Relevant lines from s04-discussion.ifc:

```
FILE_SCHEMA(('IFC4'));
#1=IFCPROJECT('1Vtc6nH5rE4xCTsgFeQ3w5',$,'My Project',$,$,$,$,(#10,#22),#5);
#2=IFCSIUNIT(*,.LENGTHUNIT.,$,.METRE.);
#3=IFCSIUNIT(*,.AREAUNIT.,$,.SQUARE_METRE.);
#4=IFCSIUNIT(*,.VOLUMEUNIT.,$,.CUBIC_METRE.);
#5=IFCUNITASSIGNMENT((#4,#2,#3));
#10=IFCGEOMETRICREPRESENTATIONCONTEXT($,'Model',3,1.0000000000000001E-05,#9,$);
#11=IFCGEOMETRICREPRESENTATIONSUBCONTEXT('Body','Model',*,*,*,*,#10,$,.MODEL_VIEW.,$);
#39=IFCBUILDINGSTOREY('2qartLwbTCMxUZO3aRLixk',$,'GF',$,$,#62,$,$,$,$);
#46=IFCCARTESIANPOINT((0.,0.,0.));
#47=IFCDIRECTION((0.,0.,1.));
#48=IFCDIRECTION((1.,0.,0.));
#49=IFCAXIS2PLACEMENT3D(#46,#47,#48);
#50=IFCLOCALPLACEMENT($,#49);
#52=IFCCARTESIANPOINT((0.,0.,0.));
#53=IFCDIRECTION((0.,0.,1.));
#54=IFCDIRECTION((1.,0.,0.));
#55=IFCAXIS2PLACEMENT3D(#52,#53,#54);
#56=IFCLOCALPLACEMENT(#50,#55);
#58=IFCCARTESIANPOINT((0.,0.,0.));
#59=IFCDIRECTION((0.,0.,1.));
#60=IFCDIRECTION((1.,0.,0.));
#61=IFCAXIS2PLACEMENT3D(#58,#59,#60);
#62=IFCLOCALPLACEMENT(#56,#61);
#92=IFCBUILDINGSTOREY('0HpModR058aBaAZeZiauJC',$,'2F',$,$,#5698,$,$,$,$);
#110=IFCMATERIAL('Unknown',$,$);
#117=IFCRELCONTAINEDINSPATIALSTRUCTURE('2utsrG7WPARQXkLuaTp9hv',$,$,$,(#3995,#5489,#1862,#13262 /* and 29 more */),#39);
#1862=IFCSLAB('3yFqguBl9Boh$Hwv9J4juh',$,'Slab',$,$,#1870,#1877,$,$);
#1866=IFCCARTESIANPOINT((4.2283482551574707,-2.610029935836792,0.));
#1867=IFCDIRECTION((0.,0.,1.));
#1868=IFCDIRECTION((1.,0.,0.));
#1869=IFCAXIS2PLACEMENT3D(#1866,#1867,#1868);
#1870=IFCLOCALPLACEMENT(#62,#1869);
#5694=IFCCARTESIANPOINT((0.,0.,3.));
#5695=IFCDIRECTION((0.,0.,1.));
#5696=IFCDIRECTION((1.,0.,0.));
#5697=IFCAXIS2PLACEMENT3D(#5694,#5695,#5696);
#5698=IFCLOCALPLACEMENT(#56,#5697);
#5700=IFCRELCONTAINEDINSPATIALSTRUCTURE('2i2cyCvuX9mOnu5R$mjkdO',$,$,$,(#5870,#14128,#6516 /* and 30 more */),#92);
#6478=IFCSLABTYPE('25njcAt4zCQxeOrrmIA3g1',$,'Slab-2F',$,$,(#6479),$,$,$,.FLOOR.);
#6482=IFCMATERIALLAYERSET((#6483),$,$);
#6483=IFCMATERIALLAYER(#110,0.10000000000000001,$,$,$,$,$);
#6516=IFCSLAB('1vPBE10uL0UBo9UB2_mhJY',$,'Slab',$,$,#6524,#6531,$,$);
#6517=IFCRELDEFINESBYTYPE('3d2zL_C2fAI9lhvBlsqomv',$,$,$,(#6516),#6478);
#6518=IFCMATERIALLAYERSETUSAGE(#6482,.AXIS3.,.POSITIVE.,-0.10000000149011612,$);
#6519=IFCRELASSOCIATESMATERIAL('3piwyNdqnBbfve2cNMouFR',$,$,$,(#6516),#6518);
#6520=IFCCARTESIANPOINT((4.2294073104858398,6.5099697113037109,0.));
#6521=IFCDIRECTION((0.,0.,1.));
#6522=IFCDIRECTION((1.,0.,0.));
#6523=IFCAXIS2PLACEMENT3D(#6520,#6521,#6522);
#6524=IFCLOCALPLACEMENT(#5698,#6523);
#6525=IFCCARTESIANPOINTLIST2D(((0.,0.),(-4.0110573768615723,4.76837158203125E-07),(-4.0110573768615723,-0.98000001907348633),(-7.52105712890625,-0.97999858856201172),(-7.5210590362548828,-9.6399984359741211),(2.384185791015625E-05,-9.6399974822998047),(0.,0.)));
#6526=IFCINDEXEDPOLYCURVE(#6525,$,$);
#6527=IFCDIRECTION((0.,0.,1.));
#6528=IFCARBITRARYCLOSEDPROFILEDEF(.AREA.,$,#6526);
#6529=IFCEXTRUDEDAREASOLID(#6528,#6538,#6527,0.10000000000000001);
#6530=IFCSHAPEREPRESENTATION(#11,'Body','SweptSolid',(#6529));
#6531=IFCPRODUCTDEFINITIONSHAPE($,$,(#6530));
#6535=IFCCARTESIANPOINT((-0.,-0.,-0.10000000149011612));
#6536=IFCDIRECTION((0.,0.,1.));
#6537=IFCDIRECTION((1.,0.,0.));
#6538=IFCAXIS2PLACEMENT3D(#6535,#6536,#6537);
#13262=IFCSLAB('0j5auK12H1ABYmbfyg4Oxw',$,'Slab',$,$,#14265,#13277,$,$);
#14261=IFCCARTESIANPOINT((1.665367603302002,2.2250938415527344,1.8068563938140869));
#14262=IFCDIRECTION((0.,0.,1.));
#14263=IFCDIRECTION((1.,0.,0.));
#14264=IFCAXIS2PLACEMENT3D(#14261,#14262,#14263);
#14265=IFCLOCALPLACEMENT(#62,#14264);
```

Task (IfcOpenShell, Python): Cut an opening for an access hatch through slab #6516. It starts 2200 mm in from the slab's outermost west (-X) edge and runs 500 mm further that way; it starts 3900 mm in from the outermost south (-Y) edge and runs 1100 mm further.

```python
import numpy as np
import ifcopenshell
import ifcopenshell.api.feature
import ifcopenshell.api.geometry
import ifcopenshell.api.root
import ifcopenshell.geom
import ifcopenshell.util.placement
import ifcopenshell.util.representation
import ifcopenshell.util.shape
import ifcopenshell.util.unit

model = ifcopenshell.open("s04-discussion.ifc")
unit_scale = ifcopenshell.util.unit.calculate_unit_scale(model)
settings = ifcopenshell.geom.settings()


def volume(element):
    """Net volume in cubic metres, openings subtracted."""
    shape = ifcopenshell.geom.create_shape(settings, element)
    return ifcopenshell.util.shape.get_volume(shape.geometry)


slab = model.by_id(6516)
before = volume(slab)

# Extent in the slab's own axes, in metres. The edges named are its -X and -Y sides.
slab_shape = ifcopenshell.geom.create_shape(settings, slab)
vertices = ifcopenshell.util.shape.get_vertices(slab_shape.geometry)
x_min, y_min, bottom = vertices.min(axis=0)
top = vertices[:, 2].max()

opening = ifcopenshell.api.root.create_entity(model, ifc_class="IfcOpeningElement", name="Access hatch opening", predefined_type="OPENING")
context = ifcopenshell.util.representation.get_context(model, "Model", "Body", "MODEL_VIEW")
width, depth = 0.5, 1.1
outline = [(0.0, 0.0), (width, 0.0), (width, depth), (0.0, depth), (0.0, 0.0)]
# Overshoot both faces by 50 mm so the cut is clean.
shape = ifcopenshell.api.geometry.add_slab_representation(
    model, context=context, depth=top - bottom + 0.1, polyline=outline
)
ifcopenshell.api.geometry.assign_representation(model, product=opening, representation=shape)

matrix = ifcopenshell.util.placement.get_local_placement(slab.ObjectPlacement)
matrix[:, 3] = matrix @ np.append(np.array([x_min + 2.2, y_min + 3.9, bottom - 0.05]) / unit_scale, 1.0)
ifcopenshell.api.geometry.edit_object_placement(model, product=opening, matrix=matrix, is_si=False)
ifcopenshell.api.feature.add_feature(model, feature=opening, element=slab)

after = volume(slab)

print(f"slab volume {before:.3f} -> {after:.3f} m3")

model.write("s04-discussion_edited.ifc")
```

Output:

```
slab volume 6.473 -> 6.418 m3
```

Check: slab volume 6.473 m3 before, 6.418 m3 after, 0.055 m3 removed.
